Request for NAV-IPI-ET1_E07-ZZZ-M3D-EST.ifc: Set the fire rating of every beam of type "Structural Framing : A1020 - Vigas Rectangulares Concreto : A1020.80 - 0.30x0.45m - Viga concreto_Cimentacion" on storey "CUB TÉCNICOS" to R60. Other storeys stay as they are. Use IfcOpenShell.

First a look at what the model holds.

```python
import ifcopenshell
import ifcopenshell.util.element

model = ifcopenshell.open("NAV-IPI-ET1_E07-ZZZ-M3D-EST.ifc")
print(model.schema)
storey = next(s for s in model.by_type("IfcBuildingStorey") if s.Name == "CUB TÉCNICOS")
beams = [e for e in ifcopenshell.util.element.get_decomposition(storey) if e.is_a("IfcBeam")]
seen = {}
for e in beams:
    element_type = ifcopenshell.util.element.get_type(e)
    key = (element_type.Name if element_type != e and element_type else None, ifcopenshell.util.element.get_pset(e, "Pset_BeamCommon", "FireRating"))
    seen[key] = seen.get(key, 0) + 1
for (name, value), count in sorted(seen.items(), key=str):
    print(count, "x", name, "|", value)
```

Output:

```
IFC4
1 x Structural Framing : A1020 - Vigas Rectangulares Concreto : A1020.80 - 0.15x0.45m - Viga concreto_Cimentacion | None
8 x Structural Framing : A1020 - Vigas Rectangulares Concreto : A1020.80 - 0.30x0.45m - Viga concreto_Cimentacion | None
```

```python
import ifcopenshell
import ifcopenshell.api.pset
import ifcopenshell.util.element

model = ifcopenshell.open("NAV-IPI-ET1_E07-ZZZ-M3D-EST.ifc")

storey = next(s for s in model.by_type("IfcBuildingStorey") if s.Name == "CUB TÉCNICOS")
beams = [e for e in ifcopenshell.util.element.get_decomposition(storey) if e.is_a("IfcBeam")]

count = 0
for e in beams:
    element_type = ifcopenshell.util.element.get_type(e)
    if element_type in (None, e) or element_type.Name != "Structural Framing : A1020 - Vigas Rectangulares Concreto : A1020.80 - 0.30x0.45m - Viga concreto_Cimentacion":
        continue
    # add_pset returns the element's existing set when there is one.
    pset = ifcopenshell.api.pset.add_pset(model, product=e, name="Pset_BeamCommon")
    ifcopenshell.api.pset.edit_pset(model, pset=pset, properties={"FireRating": "R60"})
    count += 1

print(count, "beams updated")

model.write("NAV-IPI-ET1_E07-ZZZ-M3D-EST_edited.ifc")
```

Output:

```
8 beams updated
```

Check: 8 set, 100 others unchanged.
